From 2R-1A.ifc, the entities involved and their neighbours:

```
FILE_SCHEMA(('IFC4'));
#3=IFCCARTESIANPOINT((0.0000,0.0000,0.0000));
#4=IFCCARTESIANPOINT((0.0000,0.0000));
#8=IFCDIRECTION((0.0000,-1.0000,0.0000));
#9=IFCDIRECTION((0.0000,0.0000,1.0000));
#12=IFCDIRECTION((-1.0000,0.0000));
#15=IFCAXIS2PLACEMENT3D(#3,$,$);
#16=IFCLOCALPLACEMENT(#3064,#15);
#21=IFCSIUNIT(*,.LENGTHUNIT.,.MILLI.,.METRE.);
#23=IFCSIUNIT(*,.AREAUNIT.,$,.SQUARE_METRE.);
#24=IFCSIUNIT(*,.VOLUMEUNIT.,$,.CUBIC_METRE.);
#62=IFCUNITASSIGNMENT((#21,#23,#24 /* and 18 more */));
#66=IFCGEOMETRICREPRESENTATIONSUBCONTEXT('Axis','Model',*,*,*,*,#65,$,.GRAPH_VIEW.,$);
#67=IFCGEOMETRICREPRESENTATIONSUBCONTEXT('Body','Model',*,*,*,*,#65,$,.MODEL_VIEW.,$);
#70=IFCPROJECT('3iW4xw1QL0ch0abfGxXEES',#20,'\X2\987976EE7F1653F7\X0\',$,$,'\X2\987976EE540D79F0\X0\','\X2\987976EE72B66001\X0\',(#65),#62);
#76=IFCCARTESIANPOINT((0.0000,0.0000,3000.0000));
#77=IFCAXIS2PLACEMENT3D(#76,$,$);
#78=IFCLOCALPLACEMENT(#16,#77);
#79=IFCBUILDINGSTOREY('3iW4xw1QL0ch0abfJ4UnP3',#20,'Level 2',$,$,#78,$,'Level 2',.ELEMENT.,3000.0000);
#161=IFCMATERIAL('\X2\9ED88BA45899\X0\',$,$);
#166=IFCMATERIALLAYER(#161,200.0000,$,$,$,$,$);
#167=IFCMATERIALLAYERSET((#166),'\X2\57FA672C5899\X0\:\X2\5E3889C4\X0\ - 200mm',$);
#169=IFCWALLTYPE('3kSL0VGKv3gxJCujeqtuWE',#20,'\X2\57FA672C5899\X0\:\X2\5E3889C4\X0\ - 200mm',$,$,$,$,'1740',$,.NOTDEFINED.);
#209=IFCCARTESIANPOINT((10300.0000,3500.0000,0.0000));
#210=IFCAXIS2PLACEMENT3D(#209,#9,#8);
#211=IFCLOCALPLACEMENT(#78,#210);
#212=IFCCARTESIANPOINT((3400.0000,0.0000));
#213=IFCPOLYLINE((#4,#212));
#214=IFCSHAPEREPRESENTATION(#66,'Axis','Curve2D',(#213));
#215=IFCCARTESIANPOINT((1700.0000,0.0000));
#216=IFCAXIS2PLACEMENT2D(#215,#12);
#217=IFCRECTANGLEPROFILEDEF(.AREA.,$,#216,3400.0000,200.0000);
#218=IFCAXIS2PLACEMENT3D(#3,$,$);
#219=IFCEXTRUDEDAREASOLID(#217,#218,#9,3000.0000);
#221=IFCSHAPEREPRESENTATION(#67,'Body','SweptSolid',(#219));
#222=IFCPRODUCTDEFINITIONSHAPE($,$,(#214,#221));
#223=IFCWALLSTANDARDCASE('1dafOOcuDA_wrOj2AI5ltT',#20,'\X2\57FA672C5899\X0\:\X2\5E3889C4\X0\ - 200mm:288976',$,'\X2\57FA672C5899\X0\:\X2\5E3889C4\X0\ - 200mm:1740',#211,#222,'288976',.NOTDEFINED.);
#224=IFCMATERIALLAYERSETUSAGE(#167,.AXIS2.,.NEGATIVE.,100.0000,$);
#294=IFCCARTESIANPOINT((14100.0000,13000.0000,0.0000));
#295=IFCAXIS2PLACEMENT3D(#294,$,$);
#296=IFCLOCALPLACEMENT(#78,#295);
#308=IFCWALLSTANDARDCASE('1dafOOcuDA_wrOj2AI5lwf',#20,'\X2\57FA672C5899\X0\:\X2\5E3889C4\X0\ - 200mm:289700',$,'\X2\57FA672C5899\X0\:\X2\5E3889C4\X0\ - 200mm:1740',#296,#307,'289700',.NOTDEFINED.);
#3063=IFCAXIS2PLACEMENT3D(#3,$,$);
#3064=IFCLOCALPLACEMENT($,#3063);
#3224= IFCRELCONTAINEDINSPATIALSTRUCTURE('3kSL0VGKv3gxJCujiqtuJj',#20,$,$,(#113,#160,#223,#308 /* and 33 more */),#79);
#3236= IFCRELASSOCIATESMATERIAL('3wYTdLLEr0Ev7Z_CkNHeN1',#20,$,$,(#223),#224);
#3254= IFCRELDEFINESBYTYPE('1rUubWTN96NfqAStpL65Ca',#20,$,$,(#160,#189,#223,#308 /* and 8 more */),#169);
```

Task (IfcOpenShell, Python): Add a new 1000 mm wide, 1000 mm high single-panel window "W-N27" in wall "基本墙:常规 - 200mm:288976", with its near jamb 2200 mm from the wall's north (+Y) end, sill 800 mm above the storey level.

```python
import numpy as np
import ifcopenshell
import ifcopenshell.api.feature
import ifcopenshell.api.geometry
import ifcopenshell.api.root
import ifcopenshell.api.spatial
import ifcopenshell.geom
import ifcopenshell.util.element
import ifcopenshell.util.placement
import ifcopenshell.util.representation
import ifcopenshell.util.shape
import ifcopenshell.util.unit

model = ifcopenshell.open("2R-1A.ifc")
unit_scale = ifcopenshell.util.unit.calculate_unit_scale(model)
settings = ifcopenshell.geom.settings()


def volume(element):
    """Net volume in cubic metres, openings subtracted."""
    shape = ifcopenshell.geom.create_shape(settings, element)
    return ifcopenshell.util.shape.get_volume(shape.geometry)


wall = model.by_guid("1dafOOcuDA_wrOj2AI5ltT")
storey = ifcopenshell.util.element.get_container(wall, ifc_class="IfcBuildingStorey")
context = ifcopenshell.util.representation.get_context(model, "Model", "Body", "MODEL_VIEW")
before = volume(wall)

width, height, from_end, sill = 1, 1, 2.2, 0.8  # metres

# The wall runs along its own X axis, and the end named is its -X end.
wall_shape = ifcopenshell.geom.create_shape(settings, wall)
x, y, z = ifcopenshell.util.shape.get_vertices(wall_shape.geometry).T
start = x.min() + from_end
face, thickness = float(y.min()), float(y.max() - y.min())
wall_matrix = ifcopenshell.util.placement.get_local_placement(wall.ObjectPlacement)
level = ifcopenshell.util.placement.get_local_placement(storey.ObjectPlacement)[2, 3]


def in_wall(x, y):
    """Placement at x, y metres in the wall's axes, at sill height."""
    matrix = wall_matrix.copy()
    matrix[:, 3] = wall_matrix @ np.array([x / unit_scale, y / unit_scale, 0.0, 1.0])
    matrix[2, 3] = level + sill / unit_scale
    return matrix


# Opening: a box that overshoots both wall faces by 50 mm.
opening = ifcopenshell.api.root.create_entity(model, ifc_class="IfcOpeningElement", predefined_type="OPENING")
box = ifcopenshell.api.geometry.add_wall_representation(
    model, context=context, length=width, height=height, thickness=thickness + 0.1
)
ifcopenshell.api.geometry.assign_representation(model, product=opening, representation=box)
ifcopenshell.api.geometry.edit_object_placement(model, product=opening, matrix=in_wall(start, face - 0.05), is_si=False)
ifcopenshell.api.feature.add_feature(model, feature=opening, element=wall)

window = ifcopenshell.api.root.create_entity(model, ifc_class="IfcWindow", name="W-N27", predefined_type="WINDOW")
window.OverallWidth, window.OverallHeight = width / unit_scale, height / unit_scale
window.PartitioningType = "SINGLE_PANEL"
body = ifcopenshell.api.geometry.add_window_representation(
    model,
    context=context,
    overall_width=window.OverallWidth,
    overall_height=window.OverallHeight,
    partition_type="SINGLE_PANEL",
)
ifcopenshell.api.geometry.assign_representation(model, product=window, representation=body)
ifcopenshell.api.spatial.assign_container(model, products=[window], relating_structure=storey)
ifcopenshell.api.feature.add_filling(model, opening=opening, element=window)

# Centre the window in the wall's thickness.
ifcopenshell.api.geometry.edit_object_placement(model, product=window, matrix=in_wall(start, face), is_si=False)
window_shape = ifcopenshell.geom.create_shape(settings, window)
depth = ifcopenshell.util.shape.get_vertices(window_shape.geometry)[:, 1]
offset = face + thickness / 2 - (depth.min() + depth.max()) / 2
ifcopenshell.api.geometry.edit_object_placement(model, product=window, matrix=in_wall(start, offset), is_si=False)

after = volume(wall)

print(f"wall volume {before:.3f} -> {after:.3f} m3")

model.write("2R-1A_updated.ifc")
```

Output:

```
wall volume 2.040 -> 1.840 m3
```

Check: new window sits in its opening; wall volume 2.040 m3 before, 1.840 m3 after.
